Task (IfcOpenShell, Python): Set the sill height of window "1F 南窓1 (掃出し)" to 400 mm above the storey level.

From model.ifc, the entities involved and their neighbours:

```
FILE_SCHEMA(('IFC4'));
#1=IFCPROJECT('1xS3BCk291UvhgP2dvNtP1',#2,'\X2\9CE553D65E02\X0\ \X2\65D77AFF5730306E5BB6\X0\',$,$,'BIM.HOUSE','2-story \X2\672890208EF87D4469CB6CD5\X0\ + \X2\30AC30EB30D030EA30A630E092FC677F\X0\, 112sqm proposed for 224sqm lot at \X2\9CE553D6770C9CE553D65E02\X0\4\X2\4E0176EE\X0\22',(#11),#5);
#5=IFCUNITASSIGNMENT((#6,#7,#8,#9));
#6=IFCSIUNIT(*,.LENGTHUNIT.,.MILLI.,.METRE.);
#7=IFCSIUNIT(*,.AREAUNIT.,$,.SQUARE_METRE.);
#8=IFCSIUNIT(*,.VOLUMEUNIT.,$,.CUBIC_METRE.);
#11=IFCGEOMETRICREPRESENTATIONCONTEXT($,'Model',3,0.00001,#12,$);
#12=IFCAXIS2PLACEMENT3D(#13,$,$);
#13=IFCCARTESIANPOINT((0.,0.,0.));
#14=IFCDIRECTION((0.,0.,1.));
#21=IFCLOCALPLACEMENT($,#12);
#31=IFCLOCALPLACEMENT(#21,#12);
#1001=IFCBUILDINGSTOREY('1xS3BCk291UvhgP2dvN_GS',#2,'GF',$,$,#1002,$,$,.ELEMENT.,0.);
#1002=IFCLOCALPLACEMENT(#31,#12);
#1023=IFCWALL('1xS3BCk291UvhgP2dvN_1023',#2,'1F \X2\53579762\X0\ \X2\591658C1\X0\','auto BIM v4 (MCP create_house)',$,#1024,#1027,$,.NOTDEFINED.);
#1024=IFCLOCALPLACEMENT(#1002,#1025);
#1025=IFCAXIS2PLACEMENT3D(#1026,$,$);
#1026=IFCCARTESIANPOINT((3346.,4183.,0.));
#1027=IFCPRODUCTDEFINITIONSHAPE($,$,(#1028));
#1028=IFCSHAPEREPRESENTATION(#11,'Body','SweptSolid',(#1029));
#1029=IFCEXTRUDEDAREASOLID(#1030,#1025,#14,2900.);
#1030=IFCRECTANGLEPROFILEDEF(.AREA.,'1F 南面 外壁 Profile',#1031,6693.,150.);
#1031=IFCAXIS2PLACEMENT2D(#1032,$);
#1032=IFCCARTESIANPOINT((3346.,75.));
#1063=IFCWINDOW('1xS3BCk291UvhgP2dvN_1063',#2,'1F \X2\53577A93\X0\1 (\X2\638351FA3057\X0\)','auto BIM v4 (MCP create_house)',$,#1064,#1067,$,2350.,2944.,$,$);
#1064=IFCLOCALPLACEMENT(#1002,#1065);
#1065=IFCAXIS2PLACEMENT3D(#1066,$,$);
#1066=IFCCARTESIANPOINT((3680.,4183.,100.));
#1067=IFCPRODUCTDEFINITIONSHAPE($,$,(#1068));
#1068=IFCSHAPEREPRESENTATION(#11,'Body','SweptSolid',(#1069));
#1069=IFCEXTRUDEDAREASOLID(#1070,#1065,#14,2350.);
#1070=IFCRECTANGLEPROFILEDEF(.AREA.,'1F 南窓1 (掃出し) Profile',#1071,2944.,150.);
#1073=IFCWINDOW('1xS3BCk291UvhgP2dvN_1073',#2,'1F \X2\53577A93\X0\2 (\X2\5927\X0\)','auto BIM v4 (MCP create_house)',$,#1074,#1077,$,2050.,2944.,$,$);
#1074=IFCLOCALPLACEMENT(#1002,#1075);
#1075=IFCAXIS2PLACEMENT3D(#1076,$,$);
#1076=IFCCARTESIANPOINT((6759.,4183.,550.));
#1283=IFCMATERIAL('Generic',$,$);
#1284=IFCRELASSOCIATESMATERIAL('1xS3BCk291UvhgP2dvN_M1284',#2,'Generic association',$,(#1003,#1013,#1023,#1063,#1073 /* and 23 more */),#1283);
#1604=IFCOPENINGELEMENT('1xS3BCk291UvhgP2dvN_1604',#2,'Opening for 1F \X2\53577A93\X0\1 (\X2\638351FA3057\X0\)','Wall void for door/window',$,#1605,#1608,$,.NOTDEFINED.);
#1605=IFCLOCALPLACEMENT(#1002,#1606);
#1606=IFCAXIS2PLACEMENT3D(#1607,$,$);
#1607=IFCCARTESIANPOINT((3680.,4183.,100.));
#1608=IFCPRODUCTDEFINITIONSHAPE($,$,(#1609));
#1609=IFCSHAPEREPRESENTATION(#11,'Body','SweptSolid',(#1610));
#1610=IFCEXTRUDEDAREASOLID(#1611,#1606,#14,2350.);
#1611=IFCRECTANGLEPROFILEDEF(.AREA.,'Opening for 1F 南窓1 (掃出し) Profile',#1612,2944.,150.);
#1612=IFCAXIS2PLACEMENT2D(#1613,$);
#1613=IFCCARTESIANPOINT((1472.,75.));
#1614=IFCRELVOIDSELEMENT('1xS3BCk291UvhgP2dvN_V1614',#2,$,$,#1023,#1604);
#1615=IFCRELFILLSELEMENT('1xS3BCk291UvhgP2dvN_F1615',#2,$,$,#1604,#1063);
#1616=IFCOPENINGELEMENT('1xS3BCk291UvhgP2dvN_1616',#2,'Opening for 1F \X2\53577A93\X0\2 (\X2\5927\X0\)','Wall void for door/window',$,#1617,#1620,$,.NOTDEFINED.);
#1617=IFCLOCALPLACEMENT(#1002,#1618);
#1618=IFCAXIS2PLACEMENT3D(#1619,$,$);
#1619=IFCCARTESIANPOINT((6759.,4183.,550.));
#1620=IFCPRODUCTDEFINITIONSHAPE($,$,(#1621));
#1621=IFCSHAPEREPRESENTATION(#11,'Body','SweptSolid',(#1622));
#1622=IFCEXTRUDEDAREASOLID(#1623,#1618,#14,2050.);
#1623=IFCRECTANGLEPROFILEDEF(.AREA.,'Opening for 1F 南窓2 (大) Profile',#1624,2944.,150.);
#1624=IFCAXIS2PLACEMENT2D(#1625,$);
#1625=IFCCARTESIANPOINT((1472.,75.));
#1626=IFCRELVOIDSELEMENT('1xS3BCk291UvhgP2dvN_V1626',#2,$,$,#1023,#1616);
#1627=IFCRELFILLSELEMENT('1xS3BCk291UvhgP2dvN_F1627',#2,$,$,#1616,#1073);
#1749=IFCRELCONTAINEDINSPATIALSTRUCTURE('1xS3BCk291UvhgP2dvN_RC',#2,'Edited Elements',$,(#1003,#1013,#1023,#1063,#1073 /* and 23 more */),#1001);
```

```python
import numpy as np
import ifcopenshell
import ifcopenshell.api.geometry
import ifcopenshell.geom
import ifcopenshell.util.element
import ifcopenshell.util.placement
import ifcopenshell.util.shape
import ifcopenshell.util.unit

model = ifcopenshell.open("model.ifc")
unit_scale = ifcopenshell.util.unit.calculate_unit_scale(model)

window = model.by_guid("1xS3BCk291UvhgP2dvN_1063")
opening = window.FillsVoids[0].RelatingOpeningElement
storey = ifcopenshell.util.element.get_container(window, ifc_class="IfcBuildingStorey")
level = ifcopenshell.util.placement.get_local_placement(storey.ObjectPlacement)[2, 3]

# The opening's origin need not be at the sill, so measure its lowest point.
shape = ifcopenshell.geom.create_shape(ifcopenshell.geom.settings(), opening)
bottom = ifcopenshell.util.shape.get_shape_bottom_elevation(shape, shape.geometry) / unit_scale
dz = level + 400.0 - bottom

shift = np.array([0.0, 0.0, dz])
# The window is not placed relative to its opening, so move both.
for product in (opening, window):
    matrix = ifcopenshell.util.placement.get_local_placement(product.ObjectPlacement)
    matrix[:3, 3] += shift
    ifcopenshell.api.geometry.edit_object_placement(model, product=product, matrix=matrix, is_si=False)

print(f"moved by {dz * unit_scale:+.3f} m")

model.write("model_rev.ifc")
```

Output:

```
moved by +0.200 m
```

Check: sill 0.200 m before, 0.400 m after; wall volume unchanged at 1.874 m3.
